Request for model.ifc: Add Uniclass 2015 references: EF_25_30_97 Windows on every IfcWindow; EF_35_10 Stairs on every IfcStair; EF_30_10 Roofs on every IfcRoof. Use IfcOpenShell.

First a look at what the model holds.

```python
import ifcopenshell

model = ifcopenshell.open("model.ifc")
print(model.schema)
print("classifications:", [c.Name for c in model.by_type("IfcClassification")])
for ifc_class in ("IfcDoor", "IfcRoof", "IfcStair", "IfcWall", "IfcWindow"):
    print(ifc_class, len(model.by_type(ifc_class)))
```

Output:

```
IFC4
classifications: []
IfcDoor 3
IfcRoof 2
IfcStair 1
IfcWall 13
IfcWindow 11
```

```python
import ifcopenshell
import ifcopenshell.api.classification

model = ifcopenshell.open("model.ifc")

system = ifcopenshell.api.classification.add_classification(model, classification="Uniclass 2015")

codes = {
    "IfcWindow": ("EF_25_30_97", "Windows"),
    "IfcStair": ("EF_35_10", "Stairs"),
    "IfcRoof": ("EF_30_10", "Roofs"),
}
for ifc_class, (code, name) in codes.items():
    products = model.by_type(ifc_class)
    ifcopenshell.api.classification.add_reference(
        model, products=products, classification=system, identification=code, name=name
    )
    print(code, len(products))

model.write("model_updated.ifc")
```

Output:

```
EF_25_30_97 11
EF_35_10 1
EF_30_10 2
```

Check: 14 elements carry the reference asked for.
